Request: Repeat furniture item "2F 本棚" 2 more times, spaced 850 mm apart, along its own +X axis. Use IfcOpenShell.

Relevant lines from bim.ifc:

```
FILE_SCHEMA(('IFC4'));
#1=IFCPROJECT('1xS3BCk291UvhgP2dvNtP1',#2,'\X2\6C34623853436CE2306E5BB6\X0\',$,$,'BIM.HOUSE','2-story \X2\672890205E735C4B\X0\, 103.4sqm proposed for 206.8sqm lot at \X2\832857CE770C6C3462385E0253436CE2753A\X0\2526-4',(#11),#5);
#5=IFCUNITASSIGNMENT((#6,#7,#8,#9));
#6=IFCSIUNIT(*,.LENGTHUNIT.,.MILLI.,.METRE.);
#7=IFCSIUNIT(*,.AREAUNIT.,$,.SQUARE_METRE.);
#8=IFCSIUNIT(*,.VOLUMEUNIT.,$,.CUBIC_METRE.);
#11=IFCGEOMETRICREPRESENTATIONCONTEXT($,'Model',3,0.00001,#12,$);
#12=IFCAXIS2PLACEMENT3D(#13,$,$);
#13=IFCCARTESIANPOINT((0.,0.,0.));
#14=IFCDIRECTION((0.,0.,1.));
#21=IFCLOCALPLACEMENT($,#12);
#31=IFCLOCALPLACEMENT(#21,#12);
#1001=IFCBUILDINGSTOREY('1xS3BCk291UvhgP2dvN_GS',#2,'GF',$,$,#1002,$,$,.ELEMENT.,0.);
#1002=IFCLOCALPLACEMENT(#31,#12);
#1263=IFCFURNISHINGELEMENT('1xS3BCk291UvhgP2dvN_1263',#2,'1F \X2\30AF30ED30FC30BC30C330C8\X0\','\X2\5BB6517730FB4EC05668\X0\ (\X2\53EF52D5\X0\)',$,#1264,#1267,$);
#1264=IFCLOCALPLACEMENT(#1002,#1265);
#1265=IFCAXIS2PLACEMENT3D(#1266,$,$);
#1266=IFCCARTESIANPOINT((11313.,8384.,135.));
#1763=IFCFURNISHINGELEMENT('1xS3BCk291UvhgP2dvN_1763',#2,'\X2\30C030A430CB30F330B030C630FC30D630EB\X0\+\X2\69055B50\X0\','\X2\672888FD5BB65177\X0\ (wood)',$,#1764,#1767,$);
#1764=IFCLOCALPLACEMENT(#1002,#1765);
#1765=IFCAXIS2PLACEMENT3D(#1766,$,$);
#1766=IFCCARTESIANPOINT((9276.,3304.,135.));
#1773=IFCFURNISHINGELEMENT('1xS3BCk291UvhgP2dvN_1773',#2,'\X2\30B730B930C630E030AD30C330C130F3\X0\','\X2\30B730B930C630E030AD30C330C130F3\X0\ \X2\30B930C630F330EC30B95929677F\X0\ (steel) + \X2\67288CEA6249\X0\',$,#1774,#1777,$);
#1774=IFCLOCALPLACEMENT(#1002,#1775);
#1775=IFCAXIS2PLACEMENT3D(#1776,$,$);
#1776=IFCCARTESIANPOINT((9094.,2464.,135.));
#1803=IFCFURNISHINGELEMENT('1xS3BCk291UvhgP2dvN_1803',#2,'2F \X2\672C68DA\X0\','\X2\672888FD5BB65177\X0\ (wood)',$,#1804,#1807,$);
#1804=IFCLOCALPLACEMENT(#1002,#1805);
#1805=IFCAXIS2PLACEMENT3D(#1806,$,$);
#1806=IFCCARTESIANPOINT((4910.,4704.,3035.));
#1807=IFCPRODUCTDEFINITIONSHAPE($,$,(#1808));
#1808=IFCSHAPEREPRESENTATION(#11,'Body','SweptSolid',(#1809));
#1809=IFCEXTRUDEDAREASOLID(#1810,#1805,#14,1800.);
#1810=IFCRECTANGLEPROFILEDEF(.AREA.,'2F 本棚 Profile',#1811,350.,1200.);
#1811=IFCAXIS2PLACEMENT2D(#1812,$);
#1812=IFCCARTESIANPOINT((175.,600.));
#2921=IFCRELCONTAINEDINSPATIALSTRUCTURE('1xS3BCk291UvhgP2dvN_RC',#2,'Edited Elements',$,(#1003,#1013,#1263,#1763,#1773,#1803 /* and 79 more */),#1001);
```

```python
import ifcopenshell
import ifcopenshell.api.geometry
import ifcopenshell.api.root
import ifcopenshell.util.element
import ifcopenshell.util.placement
import ifcopenshell.util.unit

model = ifcopenshell.open("bim.ifc")
unit_scale = ifcopenshell.util.unit.calculate_unit_scale(model)


def reuse_history(source, copy):
    """copy_class also copies each property set's owner history, people and application; keep the originals."""
    for rel in copy.IsDefinedBy:
        if rel.is_a("IfcRelDefinesByProperties") and (history := rel.RelatingPropertyDefinition.OwnerHistory):
            rel.RelatingPropertyDefinition.OwnerHistory = source.OwnerHistory
            ifcopenshell.util.element.remove_deep2(model, history)


source = model.by_guid("1xS3BCk291UvhgP2dvN_1803")
base = ifcopenshell.util.placement.get_local_placement(source.ObjectPlacement)
step = base[:3, 0] * 0.85 / unit_scale

for i in range(1, 3):
    copy = ifcopenshell.api.root.copy_class(model, product=source)
    copy.Representation = ifcopenshell.util.element.copy_deep(
        model, source.Representation, exclude=["IfcGeometricRepresentationContext", "IfcRepresentationMap"]
    )
    reuse_history(source, copy)
    matrix = base.copy()
    matrix[:3, 3] += i * step
    print("added at", matrix[:3, 3].round(3) + 0.0)
    ifcopenshell.api.geometry.edit_object_placement(model, product=copy, matrix=matrix, is_si=False)

model.write("bim_v2.ifc")
```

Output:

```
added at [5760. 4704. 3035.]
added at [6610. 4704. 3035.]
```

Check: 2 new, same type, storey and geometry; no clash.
